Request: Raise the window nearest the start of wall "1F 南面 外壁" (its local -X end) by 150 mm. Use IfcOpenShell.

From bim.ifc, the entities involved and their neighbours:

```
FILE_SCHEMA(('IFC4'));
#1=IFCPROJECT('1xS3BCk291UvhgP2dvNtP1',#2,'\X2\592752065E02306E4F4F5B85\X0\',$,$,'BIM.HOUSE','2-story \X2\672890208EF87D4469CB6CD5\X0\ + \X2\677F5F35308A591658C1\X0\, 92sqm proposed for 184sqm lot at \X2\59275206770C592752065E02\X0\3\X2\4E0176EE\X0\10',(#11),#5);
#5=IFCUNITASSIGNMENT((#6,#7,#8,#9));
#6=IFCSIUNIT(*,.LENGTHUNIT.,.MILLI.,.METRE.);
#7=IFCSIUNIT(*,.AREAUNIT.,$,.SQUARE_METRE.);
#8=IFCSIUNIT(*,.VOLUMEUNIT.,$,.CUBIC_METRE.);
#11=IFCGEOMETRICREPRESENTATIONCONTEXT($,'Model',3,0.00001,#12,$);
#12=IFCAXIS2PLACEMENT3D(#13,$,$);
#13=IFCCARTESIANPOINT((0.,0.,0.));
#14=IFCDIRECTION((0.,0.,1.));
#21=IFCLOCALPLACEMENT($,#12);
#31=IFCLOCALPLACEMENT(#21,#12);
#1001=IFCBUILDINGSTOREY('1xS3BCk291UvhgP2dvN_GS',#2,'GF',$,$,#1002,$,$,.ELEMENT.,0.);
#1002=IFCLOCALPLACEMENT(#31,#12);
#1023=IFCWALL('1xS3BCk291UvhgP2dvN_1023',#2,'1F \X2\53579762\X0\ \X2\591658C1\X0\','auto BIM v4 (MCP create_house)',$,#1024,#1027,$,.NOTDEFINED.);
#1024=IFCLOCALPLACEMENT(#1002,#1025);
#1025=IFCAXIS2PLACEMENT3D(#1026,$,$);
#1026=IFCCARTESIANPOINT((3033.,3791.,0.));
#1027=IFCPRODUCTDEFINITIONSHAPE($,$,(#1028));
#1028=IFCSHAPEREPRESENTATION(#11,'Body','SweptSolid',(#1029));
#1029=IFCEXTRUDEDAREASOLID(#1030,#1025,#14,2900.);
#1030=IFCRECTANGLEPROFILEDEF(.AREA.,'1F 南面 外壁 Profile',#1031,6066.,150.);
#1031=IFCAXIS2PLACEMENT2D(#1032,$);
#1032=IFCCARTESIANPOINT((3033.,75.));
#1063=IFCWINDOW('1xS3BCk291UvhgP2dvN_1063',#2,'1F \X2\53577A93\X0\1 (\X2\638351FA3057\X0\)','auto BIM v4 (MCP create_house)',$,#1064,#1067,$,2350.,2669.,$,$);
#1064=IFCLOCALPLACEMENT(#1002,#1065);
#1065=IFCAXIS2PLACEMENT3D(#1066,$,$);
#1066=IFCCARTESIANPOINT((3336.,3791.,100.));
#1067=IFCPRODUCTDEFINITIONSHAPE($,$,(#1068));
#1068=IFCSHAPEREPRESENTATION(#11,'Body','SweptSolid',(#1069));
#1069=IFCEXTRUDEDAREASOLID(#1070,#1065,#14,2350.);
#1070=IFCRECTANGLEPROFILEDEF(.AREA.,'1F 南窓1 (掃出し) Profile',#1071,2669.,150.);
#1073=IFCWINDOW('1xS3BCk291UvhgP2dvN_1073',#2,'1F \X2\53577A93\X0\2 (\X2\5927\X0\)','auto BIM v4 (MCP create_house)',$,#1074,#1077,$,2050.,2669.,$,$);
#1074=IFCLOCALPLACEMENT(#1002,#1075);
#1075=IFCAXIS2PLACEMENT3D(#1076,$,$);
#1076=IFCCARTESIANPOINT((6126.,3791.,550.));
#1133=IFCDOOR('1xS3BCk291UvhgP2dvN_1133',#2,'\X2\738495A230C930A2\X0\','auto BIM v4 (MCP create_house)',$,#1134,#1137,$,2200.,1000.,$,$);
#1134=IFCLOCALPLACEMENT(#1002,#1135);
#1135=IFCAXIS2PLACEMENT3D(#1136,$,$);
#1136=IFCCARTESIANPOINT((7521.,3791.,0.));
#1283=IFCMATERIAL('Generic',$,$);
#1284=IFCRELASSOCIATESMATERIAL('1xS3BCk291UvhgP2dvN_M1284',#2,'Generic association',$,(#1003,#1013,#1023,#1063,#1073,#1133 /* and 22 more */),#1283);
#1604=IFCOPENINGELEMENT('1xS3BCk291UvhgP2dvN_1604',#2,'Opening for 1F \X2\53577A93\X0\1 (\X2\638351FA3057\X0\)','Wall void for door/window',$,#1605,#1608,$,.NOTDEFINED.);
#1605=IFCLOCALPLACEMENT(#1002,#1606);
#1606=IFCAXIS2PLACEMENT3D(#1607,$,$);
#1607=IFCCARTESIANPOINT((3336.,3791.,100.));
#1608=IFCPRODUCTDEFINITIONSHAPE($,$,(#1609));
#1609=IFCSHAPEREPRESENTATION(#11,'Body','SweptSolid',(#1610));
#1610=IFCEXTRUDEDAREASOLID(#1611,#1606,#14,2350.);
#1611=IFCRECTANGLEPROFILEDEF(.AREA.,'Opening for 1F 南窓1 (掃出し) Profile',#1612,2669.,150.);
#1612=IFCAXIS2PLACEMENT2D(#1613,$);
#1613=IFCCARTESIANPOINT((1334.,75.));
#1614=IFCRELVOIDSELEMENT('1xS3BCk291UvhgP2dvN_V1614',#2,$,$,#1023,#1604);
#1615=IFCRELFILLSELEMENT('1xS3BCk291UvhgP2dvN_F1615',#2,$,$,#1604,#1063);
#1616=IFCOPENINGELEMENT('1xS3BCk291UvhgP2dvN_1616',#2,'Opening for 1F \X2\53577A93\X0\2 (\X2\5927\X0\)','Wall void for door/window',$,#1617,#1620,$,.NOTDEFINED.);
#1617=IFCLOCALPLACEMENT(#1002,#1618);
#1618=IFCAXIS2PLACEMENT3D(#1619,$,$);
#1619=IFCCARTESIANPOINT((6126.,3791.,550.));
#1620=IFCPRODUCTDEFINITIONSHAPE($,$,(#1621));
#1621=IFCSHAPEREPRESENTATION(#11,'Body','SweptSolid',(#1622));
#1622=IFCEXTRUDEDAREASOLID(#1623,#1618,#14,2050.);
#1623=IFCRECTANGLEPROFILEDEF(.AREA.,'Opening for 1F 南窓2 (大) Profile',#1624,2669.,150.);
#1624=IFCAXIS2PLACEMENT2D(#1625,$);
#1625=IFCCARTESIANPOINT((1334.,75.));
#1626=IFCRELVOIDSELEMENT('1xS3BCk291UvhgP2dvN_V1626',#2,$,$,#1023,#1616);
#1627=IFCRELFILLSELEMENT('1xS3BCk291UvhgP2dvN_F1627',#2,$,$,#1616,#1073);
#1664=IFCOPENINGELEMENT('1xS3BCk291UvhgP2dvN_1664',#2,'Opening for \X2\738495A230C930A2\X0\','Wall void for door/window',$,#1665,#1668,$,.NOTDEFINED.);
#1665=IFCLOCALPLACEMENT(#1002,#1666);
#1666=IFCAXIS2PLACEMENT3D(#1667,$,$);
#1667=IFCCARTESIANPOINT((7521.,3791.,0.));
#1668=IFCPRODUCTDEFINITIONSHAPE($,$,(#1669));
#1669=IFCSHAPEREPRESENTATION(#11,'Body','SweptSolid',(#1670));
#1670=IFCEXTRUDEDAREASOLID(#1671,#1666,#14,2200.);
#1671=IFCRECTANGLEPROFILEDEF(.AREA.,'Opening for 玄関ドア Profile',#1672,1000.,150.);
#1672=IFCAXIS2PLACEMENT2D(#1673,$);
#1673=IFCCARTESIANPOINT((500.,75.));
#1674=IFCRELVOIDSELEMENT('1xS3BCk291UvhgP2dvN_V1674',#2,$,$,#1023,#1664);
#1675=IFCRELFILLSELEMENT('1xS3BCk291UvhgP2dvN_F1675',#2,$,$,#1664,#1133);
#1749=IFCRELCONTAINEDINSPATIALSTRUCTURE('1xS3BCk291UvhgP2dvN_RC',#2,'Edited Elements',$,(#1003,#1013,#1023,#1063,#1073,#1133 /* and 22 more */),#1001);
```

```python
import numpy as np
import ifcopenshell
import ifcopenshell.api.geometry
import ifcopenshell.util.placement
import ifcopenshell.util.unit

model = ifcopenshell.open("bim.ifc")
unit_scale = ifcopenshell.util.unit.calculate_unit_scale(model)

window = model.by_guid("1xS3BCk291UvhgP2dvN_1063")
opening = window.FillsVoids[0].RelatingOpeningElement
dz = 150.0

shift = np.array([0.0, 0.0, dz])
# The window is not placed relative to its opening, so move both.
for product in (opening, window):
    matrix = ifcopenshell.util.placement.get_local_placement(product.ObjectPlacement)
    matrix[:3, 3] += shift
    ifcopenshell.api.geometry.edit_object_placement(model, product=product, matrix=matrix, is_si=False)

print(f"moved by {dz * unit_scale:+.3f} m")

model.write("bim-out.ifc")
```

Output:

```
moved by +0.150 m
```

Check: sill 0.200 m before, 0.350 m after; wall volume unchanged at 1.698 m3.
